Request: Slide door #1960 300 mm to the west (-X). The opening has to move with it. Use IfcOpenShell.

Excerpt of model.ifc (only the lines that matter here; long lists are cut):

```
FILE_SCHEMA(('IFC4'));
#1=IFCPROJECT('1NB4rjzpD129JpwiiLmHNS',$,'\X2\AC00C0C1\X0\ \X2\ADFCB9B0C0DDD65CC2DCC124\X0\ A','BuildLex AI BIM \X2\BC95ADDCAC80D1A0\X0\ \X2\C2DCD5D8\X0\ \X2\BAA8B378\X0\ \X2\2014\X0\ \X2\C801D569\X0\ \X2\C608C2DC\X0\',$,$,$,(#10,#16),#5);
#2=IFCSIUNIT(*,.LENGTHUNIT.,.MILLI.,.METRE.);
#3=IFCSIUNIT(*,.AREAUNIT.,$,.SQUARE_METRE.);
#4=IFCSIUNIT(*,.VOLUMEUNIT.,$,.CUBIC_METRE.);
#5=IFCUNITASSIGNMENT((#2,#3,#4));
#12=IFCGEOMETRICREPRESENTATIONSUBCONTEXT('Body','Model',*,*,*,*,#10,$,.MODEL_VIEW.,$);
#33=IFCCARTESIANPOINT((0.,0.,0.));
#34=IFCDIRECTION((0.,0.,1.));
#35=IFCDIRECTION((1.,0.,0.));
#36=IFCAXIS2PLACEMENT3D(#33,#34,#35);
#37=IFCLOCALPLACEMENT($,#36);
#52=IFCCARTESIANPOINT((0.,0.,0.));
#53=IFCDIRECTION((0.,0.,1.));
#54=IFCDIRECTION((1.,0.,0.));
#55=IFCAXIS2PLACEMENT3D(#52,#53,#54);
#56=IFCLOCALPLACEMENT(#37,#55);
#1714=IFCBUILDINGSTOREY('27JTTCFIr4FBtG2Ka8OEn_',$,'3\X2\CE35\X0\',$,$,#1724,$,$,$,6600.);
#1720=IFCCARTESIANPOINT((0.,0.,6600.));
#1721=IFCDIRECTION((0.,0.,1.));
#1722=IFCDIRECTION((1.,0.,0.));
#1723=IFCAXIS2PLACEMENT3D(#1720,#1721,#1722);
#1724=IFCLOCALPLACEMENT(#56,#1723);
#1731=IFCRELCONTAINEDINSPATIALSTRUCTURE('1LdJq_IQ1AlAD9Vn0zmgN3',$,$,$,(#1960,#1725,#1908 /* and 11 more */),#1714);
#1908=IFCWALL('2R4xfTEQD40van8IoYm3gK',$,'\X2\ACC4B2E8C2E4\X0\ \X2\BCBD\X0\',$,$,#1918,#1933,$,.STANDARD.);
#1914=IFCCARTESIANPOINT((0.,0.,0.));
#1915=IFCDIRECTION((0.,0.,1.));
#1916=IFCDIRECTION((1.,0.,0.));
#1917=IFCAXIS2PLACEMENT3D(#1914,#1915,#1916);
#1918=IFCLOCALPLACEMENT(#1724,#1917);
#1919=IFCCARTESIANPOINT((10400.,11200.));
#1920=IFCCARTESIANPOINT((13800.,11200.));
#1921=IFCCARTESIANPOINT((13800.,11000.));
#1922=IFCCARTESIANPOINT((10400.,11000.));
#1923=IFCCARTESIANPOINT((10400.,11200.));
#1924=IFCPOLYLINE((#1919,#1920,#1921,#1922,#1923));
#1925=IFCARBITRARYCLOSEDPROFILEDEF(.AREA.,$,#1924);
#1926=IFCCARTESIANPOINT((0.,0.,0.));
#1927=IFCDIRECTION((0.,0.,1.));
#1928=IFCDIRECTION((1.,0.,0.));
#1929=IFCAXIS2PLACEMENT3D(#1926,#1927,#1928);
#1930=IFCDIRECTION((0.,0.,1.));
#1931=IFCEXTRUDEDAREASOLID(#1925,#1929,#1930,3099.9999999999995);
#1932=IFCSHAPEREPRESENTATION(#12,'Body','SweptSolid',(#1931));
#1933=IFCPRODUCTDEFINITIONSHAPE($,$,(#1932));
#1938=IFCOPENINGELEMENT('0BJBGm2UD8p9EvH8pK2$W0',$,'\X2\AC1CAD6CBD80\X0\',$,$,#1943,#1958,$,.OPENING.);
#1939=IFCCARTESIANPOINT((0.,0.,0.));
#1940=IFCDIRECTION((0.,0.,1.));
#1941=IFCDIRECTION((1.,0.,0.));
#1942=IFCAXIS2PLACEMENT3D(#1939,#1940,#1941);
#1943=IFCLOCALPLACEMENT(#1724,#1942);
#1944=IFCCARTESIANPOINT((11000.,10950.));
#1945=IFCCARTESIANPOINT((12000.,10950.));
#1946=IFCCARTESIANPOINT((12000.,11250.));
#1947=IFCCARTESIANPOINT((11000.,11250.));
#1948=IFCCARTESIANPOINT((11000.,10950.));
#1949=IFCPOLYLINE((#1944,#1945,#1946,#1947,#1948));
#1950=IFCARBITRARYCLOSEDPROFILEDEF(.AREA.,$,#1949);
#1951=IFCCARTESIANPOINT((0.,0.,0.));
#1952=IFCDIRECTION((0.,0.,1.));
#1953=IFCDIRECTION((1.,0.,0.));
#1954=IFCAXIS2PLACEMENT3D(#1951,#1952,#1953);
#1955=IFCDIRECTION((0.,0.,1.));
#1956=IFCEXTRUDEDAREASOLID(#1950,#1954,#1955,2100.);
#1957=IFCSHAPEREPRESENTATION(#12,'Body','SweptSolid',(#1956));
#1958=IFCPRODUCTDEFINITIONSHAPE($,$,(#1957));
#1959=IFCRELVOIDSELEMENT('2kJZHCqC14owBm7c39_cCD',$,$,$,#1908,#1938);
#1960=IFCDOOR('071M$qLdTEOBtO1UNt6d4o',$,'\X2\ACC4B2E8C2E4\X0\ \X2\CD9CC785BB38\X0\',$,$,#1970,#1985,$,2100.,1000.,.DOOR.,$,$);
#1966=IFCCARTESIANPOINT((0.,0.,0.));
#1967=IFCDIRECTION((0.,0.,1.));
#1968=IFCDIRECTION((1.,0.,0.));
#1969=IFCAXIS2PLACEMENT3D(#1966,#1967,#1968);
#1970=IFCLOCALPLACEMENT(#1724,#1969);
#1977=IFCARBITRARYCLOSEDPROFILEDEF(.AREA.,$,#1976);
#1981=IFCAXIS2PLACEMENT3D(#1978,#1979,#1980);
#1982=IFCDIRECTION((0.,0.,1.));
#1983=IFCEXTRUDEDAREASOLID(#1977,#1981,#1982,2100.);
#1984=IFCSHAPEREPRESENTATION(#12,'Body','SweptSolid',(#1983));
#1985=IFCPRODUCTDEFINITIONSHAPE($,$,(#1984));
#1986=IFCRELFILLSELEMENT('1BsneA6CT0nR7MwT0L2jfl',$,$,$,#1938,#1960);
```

```python
import ifcopenshell
import ifcopenshell.api.geometry
import ifcopenshell.util.placement
import ifcopenshell.util.unit

model = ifcopenshell.open("model.ifc")
unit_scale = ifcopenshell.util.unit.calculate_unit_scale(model)

door = model.by_guid("071M$qLdTEOBtO1UNt6d4o")
opening = door.FillsVoids[0].RelatingOpeningElement
wall = opening.VoidsElements[0].RelatingBuildingElement

wall_matrix = ifcopenshell.util.placement.get_local_placement(wall.ObjectPlacement)
shift = wall_matrix[:3, 0] * -0.3 / unit_scale
before = ifcopenshell.util.placement.get_local_placement(door.ObjectPlacement)[:3, 3].copy()

# The door is not placed relative to its opening, so move both.
for product in (opening, door):
    matrix = ifcopenshell.util.placement.get_local_placement(product.ObjectPlacement)
    matrix[:3, 3] += shift
    ifcopenshell.api.geometry.edit_object_placement(model, product=product, matrix=matrix, is_si=False)

after = ifcopenshell.util.placement.get_local_placement(door.ObjectPlacement)[:3, 3]
print("door moved by", (after - before).round(3) + 0.0)

model.write("model_updated.ifc")
```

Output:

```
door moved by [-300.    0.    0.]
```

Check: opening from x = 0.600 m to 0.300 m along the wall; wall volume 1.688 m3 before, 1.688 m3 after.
